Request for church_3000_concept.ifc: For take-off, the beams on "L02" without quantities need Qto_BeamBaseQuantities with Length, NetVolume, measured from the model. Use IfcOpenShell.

First a look at what the model holds.

```python
import ifcopenshell
import ifcopenshell.util.element
import ifcopenshell.util.unit

model = ifcopenshell.open("church_3000_concept.ifc")
print(model.schema)
for unit_type in ("LENGTHUNIT", "AREAUNIT", "VOLUMEUNIT"):
    print(unit_type, ifcopenshell.util.unit.calculate_unit_scale(model, unit_type))
storey = next(s for s in model.by_type("IfcBuildingStorey") if s.Name == "L02")
beams = [e for e in ifcopenshell.util.element.get_decomposition(storey) if e.is_a("IfcBeam")]
for e in sorted(beams, key=lambda e: e.id()):
    print(e.id(), e.is_a(), e.Name, list(ifcopenshell.util.element.get_psets(e, qtos_only=True)), sep=" | ")
```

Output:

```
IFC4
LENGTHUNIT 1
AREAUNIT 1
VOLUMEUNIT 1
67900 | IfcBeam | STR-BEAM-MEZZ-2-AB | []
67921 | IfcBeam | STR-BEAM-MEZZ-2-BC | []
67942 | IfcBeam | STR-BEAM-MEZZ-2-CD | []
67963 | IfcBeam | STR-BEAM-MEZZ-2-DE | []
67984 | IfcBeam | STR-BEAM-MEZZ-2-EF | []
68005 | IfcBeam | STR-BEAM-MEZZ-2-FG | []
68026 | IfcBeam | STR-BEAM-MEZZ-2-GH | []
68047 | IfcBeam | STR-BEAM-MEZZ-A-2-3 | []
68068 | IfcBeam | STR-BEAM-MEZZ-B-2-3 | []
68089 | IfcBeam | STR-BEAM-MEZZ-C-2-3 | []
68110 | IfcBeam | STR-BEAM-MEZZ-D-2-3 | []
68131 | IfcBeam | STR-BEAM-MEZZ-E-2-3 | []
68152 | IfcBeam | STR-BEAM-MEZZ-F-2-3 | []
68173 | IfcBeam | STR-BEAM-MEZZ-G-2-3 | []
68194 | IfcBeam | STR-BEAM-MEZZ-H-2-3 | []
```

```python
import ifcopenshell
import ifcopenshell.api.pset
import ifcopenshell.geom
import ifcopenshell.util.element
import ifcopenshell.util.shape
import ifcopenshell.util.unit

model = ifcopenshell.open("church_3000_concept.ifc")
unit_scale = ifcopenshell.util.unit.calculate_unit_scale(model)
volume_scale = ifcopenshell.util.unit.calculate_unit_scale(model, "VOLUMEUNIT")
settings = ifcopenshell.geom.settings()

storey = next(s for s in model.by_type("IfcBuildingStorey") if s.Name == "L02")
beams = [e for e in ifcopenshell.util.element.get_decomposition(storey) if e.is_a("IfcBeam")]

for e in sorted(beams, key=lambda e: e.id()):
    if ifcopenshell.util.element.get_psets(e, qtos_only=True, should_inherit=False):
        continue
    # Geometry comes back in metres, in the element's own axes.
    shape = ifcopenshell.geom.create_shape(settings, e)
    values = {
        "Length": ifcopenshell.util.shape.get_max_xyz(shape.geometry) / unit_scale,
        "NetVolume": ifcopenshell.util.shape.get_volume(shape.geometry) / volume_scale,
    }
    qto = ifcopenshell.api.pset.add_qto(model, product=e, name="Qto_BeamBaseQuantities")
    ifcopenshell.api.pset.edit_qto(model, qto=qto, properties=values)
    print(e.id(), {k: round(v, 3) for k, v in values.items()})

model.write("church_3000_concept_rev.ifc")
```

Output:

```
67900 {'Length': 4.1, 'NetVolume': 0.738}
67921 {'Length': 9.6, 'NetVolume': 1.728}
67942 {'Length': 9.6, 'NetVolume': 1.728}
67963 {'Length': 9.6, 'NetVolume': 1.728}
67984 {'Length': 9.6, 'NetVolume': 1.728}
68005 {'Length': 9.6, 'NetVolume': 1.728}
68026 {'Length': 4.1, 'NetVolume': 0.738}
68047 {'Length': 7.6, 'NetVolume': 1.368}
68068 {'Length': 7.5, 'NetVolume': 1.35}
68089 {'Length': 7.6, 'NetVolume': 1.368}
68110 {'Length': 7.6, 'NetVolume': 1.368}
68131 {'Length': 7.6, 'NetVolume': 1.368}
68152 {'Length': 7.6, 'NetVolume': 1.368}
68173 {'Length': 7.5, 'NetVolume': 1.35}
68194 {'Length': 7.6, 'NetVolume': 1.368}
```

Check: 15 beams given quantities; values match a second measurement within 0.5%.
